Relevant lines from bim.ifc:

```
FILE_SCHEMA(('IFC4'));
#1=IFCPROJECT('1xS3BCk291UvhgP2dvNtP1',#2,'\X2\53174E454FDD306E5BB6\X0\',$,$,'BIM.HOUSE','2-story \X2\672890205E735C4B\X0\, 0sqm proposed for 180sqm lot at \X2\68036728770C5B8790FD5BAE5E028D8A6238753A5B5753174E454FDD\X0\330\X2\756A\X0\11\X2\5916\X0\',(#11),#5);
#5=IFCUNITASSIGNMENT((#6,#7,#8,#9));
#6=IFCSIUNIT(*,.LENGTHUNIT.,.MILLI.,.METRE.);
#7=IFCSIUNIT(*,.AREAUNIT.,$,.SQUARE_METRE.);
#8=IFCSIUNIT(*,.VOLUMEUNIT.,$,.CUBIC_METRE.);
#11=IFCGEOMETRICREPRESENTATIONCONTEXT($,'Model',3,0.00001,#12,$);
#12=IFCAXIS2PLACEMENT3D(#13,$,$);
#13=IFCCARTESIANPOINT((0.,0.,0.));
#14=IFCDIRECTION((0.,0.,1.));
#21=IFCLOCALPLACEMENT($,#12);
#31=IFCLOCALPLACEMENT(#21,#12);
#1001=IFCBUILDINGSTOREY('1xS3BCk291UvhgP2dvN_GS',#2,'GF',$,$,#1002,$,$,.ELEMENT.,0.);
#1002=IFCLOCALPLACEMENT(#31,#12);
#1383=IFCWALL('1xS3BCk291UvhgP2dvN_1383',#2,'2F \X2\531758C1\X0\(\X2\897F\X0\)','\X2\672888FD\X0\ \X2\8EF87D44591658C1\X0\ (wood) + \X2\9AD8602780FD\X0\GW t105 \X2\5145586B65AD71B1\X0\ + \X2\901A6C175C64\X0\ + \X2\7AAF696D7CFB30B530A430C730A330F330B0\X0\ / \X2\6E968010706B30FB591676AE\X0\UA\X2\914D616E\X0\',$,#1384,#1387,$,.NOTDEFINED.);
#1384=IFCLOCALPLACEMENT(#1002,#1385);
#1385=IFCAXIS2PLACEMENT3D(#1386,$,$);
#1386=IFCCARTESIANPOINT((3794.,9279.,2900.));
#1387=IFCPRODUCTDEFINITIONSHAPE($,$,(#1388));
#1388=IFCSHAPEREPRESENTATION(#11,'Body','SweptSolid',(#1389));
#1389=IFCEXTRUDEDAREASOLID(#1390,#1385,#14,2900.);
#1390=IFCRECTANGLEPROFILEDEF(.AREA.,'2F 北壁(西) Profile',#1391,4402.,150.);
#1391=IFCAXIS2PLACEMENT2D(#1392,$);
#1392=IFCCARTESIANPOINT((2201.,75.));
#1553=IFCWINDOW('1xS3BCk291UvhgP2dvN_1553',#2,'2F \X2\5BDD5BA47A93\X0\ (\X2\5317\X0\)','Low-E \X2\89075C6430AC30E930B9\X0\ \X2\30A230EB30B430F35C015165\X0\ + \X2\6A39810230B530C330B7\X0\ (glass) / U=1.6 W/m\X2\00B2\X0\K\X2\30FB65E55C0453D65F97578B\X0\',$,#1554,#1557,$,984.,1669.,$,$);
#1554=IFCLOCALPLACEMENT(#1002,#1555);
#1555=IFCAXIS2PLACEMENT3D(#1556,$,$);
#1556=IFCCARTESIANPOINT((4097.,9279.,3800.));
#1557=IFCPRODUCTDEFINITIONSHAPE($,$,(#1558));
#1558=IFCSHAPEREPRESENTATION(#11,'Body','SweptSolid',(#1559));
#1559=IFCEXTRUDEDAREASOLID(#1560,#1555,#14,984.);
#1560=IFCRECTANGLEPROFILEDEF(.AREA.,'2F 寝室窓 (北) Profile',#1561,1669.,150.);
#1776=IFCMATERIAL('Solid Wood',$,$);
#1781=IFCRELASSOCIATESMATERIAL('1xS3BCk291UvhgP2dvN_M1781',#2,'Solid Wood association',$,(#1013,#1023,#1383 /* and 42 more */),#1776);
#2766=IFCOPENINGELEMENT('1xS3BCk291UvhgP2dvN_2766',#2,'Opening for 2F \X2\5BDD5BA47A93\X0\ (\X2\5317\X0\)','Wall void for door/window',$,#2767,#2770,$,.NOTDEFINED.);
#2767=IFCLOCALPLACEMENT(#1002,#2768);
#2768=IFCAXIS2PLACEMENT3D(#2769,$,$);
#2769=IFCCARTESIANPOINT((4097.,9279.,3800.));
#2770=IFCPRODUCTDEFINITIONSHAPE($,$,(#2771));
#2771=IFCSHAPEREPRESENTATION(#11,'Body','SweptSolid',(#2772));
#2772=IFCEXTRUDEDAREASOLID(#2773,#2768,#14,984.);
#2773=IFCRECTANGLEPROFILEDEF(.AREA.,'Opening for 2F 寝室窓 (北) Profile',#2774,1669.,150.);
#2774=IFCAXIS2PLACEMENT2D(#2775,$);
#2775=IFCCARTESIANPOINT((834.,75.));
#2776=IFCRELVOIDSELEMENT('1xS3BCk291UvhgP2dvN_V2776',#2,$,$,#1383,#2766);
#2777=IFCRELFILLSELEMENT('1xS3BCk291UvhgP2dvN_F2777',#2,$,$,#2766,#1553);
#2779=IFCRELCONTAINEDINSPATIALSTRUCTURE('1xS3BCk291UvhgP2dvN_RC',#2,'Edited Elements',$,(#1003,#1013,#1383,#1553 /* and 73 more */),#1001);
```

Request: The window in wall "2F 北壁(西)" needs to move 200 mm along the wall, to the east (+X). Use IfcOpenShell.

```python
import ifcopenshell
import ifcopenshell.api.geometry
import ifcopenshell.util.placement

model = ifcopenshell.open("bim.ifc")

window = model.by_guid("1xS3BCk291UvhgP2dvN_1553")
opening = window.FillsVoids[0].RelatingOpeningElement
wall = opening.VoidsElements[0].RelatingBuildingElement

wall_matrix = ifcopenshell.util.placement.get_local_placement(wall.ObjectPlacement)
shift = wall_matrix[:3, 0] * 200.0
before = ifcopenshell.util.placement.get_local_placement(window.ObjectPlacement)[:3, 3].copy()

# The window is not placed relative to its opening, so move both.
for product in (opening, window):
    matrix = ifcopenshell.util.placement.get_local_placement(product.ObjectPlacement)
    matrix[:3, 3] += shift
    ifcopenshell.api.geometry.edit_object_placement(model, product=product, matrix=matrix, is_si=False)

after = ifcopenshell.util.placement.get_local_placement(window.ObjectPlacement)[:3, 3]
print("window moved by", (after - before).round(3) + 0.0)

model.write("bim-out.ifc")
```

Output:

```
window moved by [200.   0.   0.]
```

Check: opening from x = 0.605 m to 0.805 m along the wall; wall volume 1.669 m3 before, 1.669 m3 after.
